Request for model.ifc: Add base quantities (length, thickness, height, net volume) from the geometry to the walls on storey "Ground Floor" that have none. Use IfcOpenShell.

First a look at what the model holds.

```python
import ifcopenshell
import ifcopenshell.util.element
import ifcopenshell.util.unit

model = ifcopenshell.open("model.ifc")
print(model.schema)
for unit_type in ("LENGTHUNIT", "AREAUNIT", "VOLUMEUNIT"):
    print(unit_type, ifcopenshell.util.unit.calculate_unit_scale(model, unit_type))
storey = next(s for s in model.by_type("IfcBuildingStorey") if s.Name == "Ground Floor")
walls = [e for e in ifcopenshell.util.element.get_decomposition(storey) if e.is_a("IfcWall")]
for e in sorted(walls, key=lambda e: e.id()):
    print(e.id(), e.is_a(), e.Name, list(ifcopenshell.util.element.get_psets(e, qtos_only=True)), sep=" | ")
```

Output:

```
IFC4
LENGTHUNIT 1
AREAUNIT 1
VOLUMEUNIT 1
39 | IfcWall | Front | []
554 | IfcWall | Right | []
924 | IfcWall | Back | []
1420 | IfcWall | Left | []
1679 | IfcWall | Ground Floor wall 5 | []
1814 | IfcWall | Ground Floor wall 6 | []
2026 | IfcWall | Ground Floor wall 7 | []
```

```python
import ifcopenshell
import ifcopenshell.api.pset
import ifcopenshell.geom
import ifcopenshell.util.element
import ifcopenshell.util.shape
import ifcopenshell.util.unit

model = ifcopenshell.open("model.ifc")
unit_scale = ifcopenshell.util.unit.calculate_unit_scale(model)
volume_scale = ifcopenshell.util.unit.calculate_unit_scale(model, "VOLUMEUNIT")
settings = ifcopenshell.geom.settings()

storey = next(s for s in model.by_type("IfcBuildingStorey") if s.Name == "Ground Floor")
walls = [e for e in ifcopenshell.util.element.get_decomposition(storey) if e.is_a("IfcWall")]

for e in sorted(walls, key=lambda e: e.id()):
    if ifcopenshell.util.element.get_psets(e, qtos_only=True, should_inherit=False):
        continue
    # Geometry comes back in metres, in the element's own axes.
    shape = ifcopenshell.geom.create_shape(settings, e)
    values = {
        "Length": ifcopenshell.util.shape.get_x(shape.geometry) / unit_scale,
        "Width": ifcopenshell.util.shape.get_y(shape.geometry) / unit_scale,
        "Height": ifcopenshell.util.shape.get_z(shape.geometry) / unit_scale,
        "NetVolume": ifcopenshell.util.shape.get_volume(shape.geometry) / volume_scale,
    }
    qto = ifcopenshell.api.pset.add_qto(model, product=e, name="Qto_WallBaseQuantities")
    ifcopenshell.api.pset.edit_qto(model, qto=qto, properties=values)
    print(e.id(), {k: round(v, 3) for k, v in values.items()})

model.write("model_rev.ifc")
```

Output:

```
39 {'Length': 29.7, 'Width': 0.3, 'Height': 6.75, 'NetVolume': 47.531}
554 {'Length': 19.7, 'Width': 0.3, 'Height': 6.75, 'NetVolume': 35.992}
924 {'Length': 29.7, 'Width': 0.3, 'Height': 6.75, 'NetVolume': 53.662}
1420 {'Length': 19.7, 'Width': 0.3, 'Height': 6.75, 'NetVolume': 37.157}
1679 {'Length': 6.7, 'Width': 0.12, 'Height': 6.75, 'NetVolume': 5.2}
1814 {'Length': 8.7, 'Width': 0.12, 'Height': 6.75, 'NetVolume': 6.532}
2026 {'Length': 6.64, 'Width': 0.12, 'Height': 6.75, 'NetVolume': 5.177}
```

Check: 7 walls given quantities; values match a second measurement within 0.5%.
